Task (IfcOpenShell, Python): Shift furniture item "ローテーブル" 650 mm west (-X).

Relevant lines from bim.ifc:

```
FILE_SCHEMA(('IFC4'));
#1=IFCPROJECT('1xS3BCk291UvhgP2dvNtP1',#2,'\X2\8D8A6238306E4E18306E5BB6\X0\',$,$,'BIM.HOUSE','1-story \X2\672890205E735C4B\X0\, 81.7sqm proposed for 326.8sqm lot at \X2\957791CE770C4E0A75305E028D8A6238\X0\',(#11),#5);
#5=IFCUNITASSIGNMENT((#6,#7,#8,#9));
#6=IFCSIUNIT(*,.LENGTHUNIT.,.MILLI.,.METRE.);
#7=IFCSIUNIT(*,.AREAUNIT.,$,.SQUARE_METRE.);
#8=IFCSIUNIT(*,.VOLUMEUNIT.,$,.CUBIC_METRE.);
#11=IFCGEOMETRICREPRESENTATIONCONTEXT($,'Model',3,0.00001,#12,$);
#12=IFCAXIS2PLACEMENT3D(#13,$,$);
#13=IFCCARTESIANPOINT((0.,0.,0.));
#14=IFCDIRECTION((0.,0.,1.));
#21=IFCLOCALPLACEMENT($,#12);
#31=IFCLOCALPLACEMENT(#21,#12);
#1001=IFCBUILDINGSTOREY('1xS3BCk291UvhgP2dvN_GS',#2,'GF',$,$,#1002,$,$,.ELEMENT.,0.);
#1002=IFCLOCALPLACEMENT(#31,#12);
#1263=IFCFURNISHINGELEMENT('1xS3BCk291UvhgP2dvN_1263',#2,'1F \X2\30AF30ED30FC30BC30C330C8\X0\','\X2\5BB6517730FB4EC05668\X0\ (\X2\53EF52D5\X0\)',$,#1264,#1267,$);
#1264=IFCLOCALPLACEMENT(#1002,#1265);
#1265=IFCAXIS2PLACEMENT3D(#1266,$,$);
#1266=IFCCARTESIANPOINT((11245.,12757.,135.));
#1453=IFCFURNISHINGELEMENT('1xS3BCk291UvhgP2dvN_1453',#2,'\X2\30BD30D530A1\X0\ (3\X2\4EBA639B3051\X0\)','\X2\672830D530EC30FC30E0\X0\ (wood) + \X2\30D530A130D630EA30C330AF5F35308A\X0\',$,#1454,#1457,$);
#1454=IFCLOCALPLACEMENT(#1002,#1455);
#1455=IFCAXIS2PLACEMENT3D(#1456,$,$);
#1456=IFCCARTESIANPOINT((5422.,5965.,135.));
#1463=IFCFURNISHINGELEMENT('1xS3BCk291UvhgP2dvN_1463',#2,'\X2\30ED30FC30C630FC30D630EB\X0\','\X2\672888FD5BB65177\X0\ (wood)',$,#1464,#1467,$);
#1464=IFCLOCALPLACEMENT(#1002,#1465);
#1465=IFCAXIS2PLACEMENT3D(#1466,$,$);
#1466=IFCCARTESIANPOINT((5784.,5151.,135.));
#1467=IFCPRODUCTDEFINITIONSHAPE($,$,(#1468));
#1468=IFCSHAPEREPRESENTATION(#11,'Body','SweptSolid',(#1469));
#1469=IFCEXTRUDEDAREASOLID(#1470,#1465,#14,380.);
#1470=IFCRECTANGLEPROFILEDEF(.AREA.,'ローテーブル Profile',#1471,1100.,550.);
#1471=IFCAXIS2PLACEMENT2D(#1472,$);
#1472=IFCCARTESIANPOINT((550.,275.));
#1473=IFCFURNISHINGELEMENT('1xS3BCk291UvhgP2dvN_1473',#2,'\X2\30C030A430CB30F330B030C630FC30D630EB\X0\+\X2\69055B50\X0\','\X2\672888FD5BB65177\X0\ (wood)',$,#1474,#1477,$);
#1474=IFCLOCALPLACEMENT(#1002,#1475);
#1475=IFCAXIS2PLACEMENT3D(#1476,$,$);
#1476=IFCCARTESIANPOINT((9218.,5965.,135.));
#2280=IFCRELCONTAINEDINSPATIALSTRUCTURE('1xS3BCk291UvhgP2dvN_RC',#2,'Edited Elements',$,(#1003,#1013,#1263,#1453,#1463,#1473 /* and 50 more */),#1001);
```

```python
import ifcopenshell
import ifcopenshell.api.geometry
import ifcopenshell.util.placement

model = ifcopenshell.open("bim.ifc")

item = model.by_guid("1xS3BCk291UvhgP2dvN_1463")
matrix = ifcopenshell.util.placement.get_local_placement(item.ObjectPlacement)
matrix[0, 3] -= 650.0
ifcopenshell.api.geometry.edit_object_placement(model, product=item, matrix=matrix, is_si=False)

print(ifcopenshell.util.placement.get_local_placement(item.ObjectPlacement).round(3) + 0.0)

model.write("bim_updated.ifc")
```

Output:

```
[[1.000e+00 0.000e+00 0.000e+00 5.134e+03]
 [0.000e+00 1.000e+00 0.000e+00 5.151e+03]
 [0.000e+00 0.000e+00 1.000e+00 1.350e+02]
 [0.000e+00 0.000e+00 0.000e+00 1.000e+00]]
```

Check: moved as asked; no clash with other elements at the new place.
